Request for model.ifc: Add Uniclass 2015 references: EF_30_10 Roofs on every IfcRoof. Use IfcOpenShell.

First a look at what the model holds.

```python
import ifcopenshell

model = ifcopenshell.open("model.ifc")
print(model.schema)
print("classifications:", [c.Name for c in model.by_type("IfcClassification")])
for ifc_class in ("IfcDoor", "IfcRoof", "IfcStair", "IfcWall", "IfcWindow"):
    print(ifc_class, len(model.by_type(ifc_class)))
```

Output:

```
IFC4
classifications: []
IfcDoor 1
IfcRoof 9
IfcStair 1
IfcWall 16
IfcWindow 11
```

```python
import ifcopenshell
import ifcopenshell.api.classification

model = ifcopenshell.open("model.ifc")

system = ifcopenshell.api.classification.add_classification(model, classification="Uniclass 2015")

codes = {
    "IfcRoof": ("EF_30_10", "Roofs"),
}
for ifc_class, (code, name) in codes.items():
    products = model.by_type(ifc_class)
    ifcopenshell.api.classification.add_reference(
        model, products=products, classification=system, identification=code, name=name
    )
    print(code, len(products))

model.write("model-out.ifc")
```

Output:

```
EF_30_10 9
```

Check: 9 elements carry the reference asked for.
